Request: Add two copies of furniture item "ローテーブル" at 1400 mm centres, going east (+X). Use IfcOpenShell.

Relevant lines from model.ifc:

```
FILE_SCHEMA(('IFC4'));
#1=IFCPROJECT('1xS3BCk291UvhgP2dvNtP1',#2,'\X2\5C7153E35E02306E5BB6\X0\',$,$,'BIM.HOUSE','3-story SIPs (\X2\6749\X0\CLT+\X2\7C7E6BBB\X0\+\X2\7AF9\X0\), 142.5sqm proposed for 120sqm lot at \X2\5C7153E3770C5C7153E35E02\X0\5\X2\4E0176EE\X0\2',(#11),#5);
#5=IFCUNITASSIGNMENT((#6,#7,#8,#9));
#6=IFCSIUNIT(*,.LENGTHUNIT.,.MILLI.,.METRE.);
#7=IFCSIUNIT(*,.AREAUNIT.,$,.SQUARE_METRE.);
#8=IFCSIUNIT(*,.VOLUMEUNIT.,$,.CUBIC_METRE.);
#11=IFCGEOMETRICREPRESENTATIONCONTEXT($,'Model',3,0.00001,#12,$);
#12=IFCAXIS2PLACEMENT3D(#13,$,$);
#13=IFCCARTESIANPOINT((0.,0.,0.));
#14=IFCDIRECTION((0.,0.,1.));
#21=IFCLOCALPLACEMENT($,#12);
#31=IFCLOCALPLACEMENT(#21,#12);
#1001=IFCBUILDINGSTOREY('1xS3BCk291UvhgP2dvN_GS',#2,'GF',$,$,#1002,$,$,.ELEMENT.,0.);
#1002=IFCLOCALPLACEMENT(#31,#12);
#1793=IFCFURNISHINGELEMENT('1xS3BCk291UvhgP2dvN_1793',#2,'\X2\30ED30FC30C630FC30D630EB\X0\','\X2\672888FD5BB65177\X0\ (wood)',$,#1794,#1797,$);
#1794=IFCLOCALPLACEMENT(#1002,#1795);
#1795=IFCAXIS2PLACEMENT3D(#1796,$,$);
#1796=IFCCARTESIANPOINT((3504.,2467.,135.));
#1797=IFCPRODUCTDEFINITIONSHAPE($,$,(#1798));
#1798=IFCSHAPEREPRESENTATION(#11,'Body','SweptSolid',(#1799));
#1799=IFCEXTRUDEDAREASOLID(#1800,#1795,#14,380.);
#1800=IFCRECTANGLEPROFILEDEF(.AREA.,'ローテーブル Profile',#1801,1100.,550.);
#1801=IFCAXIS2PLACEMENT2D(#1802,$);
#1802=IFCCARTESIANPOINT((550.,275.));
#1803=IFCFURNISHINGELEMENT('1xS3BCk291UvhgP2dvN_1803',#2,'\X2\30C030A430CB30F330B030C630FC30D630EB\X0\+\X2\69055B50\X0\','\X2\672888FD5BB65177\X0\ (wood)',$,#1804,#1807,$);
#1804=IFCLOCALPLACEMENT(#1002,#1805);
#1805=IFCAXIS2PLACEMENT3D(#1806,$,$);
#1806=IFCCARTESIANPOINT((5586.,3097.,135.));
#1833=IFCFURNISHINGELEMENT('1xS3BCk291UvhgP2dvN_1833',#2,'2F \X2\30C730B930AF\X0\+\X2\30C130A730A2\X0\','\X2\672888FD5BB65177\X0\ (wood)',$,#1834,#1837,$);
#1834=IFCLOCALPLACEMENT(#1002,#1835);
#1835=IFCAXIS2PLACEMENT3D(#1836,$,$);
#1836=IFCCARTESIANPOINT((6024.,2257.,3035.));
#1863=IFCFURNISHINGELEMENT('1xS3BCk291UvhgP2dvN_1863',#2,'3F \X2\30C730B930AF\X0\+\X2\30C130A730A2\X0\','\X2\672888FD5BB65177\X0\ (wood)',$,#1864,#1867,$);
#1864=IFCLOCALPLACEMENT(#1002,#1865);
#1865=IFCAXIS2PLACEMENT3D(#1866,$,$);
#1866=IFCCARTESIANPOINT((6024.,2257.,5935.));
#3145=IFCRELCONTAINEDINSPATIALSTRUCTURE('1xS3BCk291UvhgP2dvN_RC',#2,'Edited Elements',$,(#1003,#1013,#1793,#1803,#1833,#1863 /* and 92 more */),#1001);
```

```python
import numpy as np
import ifcopenshell
import ifcopenshell.api.geometry
import ifcopenshell.api.root
import ifcopenshell.util.element
import ifcopenshell.util.placement
import ifcopenshell.util.unit

model = ifcopenshell.open("model.ifc")
unit_scale = ifcopenshell.util.unit.calculate_unit_scale(model)


def reuse_history(source, copy):
    """copy_class also copies each property set's owner history, people and application; keep the originals."""
    for rel in copy.IsDefinedBy:
        if rel.is_a("IfcRelDefinesByProperties") and (history := rel.RelatingPropertyDefinition.OwnerHistory):
            rel.RelatingPropertyDefinition.OwnerHistory = source.OwnerHistory
            ifcopenshell.util.element.remove_deep2(model, history)


source = model.by_guid("1xS3BCk291UvhgP2dvN_1793")
base = ifcopenshell.util.placement.get_local_placement(source.ObjectPlacement)
step = np.array([1.0, 0.0, 0.0]) * 1.4 / unit_scale

for i in range(1, 3):
    copy = ifcopenshell.api.root.copy_class(model, product=source)
    copy.Representation = ifcopenshell.util.element.copy_deep(
        model, source.Representation, exclude=["IfcGeometricRepresentationContext", "IfcRepresentationMap"]
    )
    reuse_history(source, copy)
    matrix = base.copy()
    matrix[:3, 3] += i * step
    print("added at", matrix[:3, 3].round(3) + 0.0)
    ifcopenshell.api.geometry.edit_object_placement(model, product=copy, matrix=matrix, is_si=False)

model.write("model_updated.ifc")
```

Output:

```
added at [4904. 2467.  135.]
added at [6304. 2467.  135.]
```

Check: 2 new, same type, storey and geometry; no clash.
